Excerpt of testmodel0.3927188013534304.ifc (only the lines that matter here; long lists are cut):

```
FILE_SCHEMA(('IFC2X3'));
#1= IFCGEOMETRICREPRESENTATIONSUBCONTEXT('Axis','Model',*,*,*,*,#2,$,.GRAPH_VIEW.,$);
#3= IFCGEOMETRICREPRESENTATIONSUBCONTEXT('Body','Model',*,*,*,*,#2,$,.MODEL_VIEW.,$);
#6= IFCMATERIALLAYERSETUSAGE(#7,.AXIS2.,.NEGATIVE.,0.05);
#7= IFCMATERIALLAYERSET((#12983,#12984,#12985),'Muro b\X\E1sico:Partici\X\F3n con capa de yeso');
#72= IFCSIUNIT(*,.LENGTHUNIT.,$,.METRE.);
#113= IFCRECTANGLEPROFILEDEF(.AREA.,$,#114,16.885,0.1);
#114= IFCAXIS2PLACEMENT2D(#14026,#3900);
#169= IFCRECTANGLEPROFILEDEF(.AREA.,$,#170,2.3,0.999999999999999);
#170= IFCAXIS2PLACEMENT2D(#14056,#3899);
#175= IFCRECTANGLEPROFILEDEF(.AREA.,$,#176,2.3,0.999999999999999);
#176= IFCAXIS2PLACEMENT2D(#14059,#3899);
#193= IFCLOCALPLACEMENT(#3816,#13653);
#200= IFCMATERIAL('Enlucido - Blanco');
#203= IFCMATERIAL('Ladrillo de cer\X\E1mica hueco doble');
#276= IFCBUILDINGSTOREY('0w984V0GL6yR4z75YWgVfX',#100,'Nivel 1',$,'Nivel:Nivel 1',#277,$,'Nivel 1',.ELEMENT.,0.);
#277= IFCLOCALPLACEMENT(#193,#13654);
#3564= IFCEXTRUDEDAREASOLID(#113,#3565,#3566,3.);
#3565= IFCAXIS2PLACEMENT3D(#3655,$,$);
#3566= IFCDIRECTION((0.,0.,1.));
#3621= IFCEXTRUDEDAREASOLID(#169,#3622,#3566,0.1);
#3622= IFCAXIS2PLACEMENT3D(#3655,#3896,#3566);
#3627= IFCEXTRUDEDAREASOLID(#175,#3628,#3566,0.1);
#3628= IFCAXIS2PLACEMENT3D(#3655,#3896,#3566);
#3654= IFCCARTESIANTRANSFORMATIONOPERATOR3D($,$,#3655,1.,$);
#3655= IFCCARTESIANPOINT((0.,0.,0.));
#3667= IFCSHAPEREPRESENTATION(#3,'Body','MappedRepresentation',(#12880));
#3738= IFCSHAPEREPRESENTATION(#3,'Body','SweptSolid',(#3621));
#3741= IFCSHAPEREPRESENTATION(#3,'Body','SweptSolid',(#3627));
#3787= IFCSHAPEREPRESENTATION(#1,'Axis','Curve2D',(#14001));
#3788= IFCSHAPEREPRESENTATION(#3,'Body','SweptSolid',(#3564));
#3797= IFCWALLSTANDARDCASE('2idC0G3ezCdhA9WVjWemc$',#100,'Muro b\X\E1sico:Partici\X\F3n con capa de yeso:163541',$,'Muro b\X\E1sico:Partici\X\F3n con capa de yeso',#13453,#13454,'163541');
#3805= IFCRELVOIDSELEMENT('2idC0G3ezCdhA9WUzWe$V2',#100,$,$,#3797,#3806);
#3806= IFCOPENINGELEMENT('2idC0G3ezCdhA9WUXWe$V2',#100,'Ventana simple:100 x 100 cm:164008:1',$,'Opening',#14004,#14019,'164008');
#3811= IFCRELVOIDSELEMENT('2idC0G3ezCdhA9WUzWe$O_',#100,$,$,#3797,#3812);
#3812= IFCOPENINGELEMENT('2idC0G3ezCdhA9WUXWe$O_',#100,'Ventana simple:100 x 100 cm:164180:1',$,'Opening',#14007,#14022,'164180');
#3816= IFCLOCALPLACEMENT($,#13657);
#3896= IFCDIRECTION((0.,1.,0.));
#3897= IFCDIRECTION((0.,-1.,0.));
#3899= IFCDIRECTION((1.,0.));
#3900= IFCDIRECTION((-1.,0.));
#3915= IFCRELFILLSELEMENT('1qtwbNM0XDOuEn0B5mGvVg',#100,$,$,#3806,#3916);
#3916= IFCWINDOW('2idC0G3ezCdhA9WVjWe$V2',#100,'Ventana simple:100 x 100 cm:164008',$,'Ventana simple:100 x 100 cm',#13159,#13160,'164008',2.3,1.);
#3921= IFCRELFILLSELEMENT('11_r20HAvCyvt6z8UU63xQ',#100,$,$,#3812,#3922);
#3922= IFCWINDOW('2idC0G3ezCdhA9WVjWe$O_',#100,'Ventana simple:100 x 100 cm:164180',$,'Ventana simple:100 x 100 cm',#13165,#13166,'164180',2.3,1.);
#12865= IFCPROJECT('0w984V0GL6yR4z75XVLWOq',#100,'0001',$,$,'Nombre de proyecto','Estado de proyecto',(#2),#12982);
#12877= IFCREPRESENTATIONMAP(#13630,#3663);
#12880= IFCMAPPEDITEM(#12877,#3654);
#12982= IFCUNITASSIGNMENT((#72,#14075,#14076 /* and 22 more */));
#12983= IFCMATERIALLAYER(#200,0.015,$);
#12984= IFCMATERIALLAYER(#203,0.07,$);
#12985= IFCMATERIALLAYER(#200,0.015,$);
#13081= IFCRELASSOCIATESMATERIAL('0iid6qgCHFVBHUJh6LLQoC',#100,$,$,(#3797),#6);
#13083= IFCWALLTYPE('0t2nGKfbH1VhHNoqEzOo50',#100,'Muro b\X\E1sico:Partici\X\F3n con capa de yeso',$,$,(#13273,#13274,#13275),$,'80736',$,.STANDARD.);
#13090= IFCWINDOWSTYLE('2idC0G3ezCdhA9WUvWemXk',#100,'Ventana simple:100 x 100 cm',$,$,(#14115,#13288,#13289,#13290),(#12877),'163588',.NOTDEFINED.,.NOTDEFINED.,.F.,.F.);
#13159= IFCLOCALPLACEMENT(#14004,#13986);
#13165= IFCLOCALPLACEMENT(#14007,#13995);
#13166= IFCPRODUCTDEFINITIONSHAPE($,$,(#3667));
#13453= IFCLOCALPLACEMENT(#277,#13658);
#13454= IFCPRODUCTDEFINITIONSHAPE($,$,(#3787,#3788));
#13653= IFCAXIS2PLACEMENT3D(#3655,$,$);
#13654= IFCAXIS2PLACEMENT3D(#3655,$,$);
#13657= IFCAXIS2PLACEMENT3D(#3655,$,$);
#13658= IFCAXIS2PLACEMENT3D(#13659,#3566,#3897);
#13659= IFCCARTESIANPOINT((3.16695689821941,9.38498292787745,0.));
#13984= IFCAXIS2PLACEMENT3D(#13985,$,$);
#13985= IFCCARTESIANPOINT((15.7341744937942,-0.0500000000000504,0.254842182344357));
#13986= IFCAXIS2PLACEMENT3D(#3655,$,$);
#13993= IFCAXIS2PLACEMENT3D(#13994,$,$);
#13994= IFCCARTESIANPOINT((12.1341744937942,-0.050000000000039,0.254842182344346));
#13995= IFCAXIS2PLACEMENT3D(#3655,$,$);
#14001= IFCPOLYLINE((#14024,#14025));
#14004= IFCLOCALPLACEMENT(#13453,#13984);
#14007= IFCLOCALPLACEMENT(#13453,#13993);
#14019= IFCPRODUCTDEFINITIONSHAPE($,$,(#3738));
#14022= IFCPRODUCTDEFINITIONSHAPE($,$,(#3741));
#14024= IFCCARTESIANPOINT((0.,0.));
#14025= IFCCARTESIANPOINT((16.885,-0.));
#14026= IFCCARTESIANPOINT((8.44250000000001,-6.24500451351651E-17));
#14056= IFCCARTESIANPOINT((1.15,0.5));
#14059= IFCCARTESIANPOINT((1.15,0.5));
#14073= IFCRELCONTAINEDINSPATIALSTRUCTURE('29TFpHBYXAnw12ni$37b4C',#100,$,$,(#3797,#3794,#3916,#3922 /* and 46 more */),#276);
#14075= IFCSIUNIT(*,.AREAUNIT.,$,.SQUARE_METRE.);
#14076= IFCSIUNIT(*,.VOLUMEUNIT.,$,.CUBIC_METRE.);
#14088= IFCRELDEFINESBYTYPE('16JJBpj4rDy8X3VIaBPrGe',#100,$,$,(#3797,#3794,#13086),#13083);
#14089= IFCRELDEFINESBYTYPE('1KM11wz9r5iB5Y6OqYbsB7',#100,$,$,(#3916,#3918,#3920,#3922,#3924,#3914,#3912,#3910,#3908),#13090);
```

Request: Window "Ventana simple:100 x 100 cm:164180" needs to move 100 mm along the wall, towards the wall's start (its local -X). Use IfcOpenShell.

```python
import ifcopenshell
import ifcopenshell.api.geometry
import ifcopenshell.util.placement

model = ifcopenshell.open("testmodel0.3927188013534304.ifc")

window = model.by_guid("2idC0G3ezCdhA9WVjWe$O_")
opening = window.FillsVoids[0].RelatingOpeningElement
wall = opening.VoidsElements[0].RelatingBuildingElement

wall_matrix = ifcopenshell.util.placement.get_local_placement(wall.ObjectPlacement)
shift = wall_matrix[:3, 0] * -0.1
before = ifcopenshell.util.placement.get_local_placement(window.ObjectPlacement)[:3, 3].copy()

# The window is placed relative to its opening, so it follows when the opening moves.
matrix = ifcopenshell.util.placement.get_local_placement(opening.ObjectPlacement)
matrix[:3, 3] += shift
ifcopenshell.api.geometry.edit_object_placement(
    model, product=opening, matrix=matrix, is_si=False, should_transform_children=True
)

after = ifcopenshell.util.placement.get_local_placement(window.ObjectPlacement)[:3, 3]
print("window moved by", (after - before).round(3) + 0.0)

model.write("testmodel0.3927188013534304-out.ifc")
```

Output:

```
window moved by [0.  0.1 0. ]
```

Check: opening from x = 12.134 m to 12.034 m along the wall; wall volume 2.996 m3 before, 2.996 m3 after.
